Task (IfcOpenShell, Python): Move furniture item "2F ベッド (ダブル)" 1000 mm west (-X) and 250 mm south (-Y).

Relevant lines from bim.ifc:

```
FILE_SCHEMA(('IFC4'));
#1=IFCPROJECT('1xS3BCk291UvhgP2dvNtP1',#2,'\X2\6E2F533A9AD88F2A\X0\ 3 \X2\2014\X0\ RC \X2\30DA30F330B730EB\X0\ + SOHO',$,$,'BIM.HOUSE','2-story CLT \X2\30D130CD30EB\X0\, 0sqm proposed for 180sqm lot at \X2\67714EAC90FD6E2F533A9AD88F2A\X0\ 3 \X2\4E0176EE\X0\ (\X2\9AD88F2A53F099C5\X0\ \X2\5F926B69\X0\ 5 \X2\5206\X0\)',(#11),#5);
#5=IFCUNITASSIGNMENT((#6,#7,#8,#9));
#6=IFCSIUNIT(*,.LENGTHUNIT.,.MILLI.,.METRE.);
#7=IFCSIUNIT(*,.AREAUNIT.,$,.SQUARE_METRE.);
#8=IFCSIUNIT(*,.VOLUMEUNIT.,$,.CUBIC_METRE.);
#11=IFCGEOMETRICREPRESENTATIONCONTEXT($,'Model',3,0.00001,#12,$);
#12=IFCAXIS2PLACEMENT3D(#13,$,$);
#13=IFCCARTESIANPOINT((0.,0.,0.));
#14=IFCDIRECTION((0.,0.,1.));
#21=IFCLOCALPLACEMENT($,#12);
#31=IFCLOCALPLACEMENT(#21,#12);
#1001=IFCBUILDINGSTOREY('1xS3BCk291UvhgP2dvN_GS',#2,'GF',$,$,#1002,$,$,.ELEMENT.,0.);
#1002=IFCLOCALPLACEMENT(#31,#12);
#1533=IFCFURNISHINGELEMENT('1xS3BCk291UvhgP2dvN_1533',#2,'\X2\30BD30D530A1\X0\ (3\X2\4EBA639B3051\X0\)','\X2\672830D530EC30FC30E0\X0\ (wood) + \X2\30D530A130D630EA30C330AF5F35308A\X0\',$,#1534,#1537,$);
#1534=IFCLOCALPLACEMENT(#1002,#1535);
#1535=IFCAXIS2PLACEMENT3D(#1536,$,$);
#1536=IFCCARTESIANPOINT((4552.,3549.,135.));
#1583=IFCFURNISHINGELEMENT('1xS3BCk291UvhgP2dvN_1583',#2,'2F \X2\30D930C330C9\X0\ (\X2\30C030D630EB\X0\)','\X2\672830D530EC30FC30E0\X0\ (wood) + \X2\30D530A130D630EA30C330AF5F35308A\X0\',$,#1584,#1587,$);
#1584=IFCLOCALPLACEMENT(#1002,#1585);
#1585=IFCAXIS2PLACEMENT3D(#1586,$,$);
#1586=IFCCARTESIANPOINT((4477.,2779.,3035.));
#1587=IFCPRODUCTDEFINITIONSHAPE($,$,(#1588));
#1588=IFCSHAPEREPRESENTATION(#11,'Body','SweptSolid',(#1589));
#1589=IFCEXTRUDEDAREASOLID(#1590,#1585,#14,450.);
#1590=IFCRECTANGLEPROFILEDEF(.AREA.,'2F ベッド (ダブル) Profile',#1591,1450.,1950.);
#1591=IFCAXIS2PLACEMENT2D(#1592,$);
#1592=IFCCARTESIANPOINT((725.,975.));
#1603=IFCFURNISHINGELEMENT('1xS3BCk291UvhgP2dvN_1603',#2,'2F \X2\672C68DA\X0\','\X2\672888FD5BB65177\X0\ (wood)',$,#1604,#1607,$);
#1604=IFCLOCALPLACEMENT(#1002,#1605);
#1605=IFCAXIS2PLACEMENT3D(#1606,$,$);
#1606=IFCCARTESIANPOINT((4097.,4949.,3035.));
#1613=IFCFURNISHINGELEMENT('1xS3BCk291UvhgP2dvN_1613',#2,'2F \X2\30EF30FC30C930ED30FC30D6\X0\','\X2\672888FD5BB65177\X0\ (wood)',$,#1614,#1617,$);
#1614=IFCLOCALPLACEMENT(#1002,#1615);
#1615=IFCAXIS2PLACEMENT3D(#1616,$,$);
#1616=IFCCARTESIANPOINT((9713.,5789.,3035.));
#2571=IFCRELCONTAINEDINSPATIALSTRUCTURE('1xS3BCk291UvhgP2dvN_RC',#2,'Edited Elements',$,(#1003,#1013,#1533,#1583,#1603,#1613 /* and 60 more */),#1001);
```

```python
import ifcopenshell
import ifcopenshell.api.geometry
import ifcopenshell.util.placement
import ifcopenshell.util.unit

model = ifcopenshell.open("bim.ifc")
unit_scale = ifcopenshell.util.unit.calculate_unit_scale(model)

item = model.by_id(1583)
matrix = ifcopenshell.util.placement.get_local_placement(item.ObjectPlacement)
matrix[0, 3] -= 1 / unit_scale
matrix[1, 3] -= 0.25 / unit_scale
ifcopenshell.api.geometry.edit_object_placement(model, product=item, matrix=matrix, is_si=False)

print(ifcopenshell.util.placement.get_local_placement(item.ObjectPlacement).round(3) + 0.0)

model.write("bim_v2.ifc")
```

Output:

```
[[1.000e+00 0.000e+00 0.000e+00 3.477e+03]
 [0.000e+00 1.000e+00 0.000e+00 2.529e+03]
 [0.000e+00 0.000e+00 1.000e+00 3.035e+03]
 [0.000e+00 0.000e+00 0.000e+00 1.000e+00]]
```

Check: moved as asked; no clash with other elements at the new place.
